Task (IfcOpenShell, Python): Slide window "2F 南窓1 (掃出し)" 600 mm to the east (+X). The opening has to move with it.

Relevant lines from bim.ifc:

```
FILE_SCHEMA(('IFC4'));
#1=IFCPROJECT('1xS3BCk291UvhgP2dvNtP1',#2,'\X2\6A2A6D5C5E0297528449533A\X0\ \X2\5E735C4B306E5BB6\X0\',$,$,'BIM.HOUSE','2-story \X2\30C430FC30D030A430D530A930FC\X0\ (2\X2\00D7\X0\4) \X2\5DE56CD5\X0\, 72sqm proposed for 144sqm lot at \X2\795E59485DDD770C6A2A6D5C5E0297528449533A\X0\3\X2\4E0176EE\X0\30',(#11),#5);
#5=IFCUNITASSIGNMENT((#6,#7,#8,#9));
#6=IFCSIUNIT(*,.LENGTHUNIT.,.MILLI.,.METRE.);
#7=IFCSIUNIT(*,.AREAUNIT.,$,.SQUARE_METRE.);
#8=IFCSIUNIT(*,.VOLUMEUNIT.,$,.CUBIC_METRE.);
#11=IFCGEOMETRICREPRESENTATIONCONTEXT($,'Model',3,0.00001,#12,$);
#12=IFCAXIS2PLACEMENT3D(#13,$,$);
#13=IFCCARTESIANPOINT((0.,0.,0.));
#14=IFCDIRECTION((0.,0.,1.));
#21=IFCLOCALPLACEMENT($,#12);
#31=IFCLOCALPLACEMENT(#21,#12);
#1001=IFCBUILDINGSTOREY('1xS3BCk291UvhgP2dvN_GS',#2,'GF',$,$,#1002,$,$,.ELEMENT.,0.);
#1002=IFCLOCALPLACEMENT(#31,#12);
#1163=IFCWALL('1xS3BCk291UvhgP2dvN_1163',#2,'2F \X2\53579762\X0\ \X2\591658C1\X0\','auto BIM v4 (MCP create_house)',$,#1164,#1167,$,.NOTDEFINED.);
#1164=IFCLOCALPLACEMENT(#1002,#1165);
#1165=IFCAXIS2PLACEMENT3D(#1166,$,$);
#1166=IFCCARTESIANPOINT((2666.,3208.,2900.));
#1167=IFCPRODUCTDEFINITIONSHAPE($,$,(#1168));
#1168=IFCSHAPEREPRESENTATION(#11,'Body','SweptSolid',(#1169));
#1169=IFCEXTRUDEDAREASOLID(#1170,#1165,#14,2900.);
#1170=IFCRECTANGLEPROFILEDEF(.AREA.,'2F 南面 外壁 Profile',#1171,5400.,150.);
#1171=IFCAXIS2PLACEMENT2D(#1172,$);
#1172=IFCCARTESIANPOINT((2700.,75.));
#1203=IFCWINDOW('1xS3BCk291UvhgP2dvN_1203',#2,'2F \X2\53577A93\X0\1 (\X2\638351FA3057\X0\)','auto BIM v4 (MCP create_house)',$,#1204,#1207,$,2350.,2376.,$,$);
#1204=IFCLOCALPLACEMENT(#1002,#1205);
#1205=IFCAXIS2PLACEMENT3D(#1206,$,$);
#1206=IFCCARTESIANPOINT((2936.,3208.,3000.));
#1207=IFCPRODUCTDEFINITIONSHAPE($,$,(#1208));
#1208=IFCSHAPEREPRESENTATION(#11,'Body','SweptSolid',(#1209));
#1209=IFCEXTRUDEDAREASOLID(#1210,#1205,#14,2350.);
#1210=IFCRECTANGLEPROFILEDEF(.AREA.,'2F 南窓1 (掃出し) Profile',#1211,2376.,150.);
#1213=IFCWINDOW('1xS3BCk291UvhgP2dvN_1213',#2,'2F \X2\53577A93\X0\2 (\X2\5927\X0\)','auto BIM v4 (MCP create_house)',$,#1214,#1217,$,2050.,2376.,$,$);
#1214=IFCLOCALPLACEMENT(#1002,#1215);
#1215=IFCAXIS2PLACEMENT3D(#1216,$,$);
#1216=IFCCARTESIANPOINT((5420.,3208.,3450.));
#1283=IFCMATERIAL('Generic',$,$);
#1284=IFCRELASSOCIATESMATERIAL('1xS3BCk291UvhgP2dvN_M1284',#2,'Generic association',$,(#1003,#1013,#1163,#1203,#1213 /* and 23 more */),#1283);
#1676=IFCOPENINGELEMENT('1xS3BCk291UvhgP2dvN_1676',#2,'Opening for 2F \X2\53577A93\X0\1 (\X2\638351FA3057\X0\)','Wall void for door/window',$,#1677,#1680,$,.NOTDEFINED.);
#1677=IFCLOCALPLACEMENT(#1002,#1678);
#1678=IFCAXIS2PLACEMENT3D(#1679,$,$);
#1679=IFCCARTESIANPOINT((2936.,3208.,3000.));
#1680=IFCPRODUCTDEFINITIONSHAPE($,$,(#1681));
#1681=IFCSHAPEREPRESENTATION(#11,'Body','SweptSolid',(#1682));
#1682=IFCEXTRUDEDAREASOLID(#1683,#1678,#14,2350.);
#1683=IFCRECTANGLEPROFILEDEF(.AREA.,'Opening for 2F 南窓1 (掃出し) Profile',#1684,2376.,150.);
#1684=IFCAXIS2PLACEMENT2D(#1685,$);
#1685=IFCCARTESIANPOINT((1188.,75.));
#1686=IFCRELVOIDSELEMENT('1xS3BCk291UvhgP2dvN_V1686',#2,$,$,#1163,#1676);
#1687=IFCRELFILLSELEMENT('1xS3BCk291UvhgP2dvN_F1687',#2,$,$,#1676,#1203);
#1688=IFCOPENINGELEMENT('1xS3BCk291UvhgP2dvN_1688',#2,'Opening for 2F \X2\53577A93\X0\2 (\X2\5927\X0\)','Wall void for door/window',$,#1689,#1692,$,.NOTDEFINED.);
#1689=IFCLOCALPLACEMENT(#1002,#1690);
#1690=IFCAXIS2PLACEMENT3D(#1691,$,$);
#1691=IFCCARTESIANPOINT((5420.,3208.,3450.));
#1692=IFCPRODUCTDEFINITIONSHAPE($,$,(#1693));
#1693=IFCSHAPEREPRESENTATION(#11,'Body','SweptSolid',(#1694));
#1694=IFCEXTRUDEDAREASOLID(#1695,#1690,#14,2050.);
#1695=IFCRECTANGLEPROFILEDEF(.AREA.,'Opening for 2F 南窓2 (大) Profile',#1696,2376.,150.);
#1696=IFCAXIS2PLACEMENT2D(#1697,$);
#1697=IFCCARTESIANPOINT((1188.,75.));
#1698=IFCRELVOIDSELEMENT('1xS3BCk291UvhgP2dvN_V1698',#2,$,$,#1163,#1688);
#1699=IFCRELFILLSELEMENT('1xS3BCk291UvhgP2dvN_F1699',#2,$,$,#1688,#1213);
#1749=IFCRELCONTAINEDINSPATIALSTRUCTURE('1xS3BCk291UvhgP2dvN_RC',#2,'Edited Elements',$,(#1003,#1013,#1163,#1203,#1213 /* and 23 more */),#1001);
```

```python
import ifcopenshell
import ifcopenshell.api.geometry
import ifcopenshell.util.placement

model = ifcopenshell.open("bim.ifc")

window = model.by_guid("1xS3BCk291UvhgP2dvN_1203")
opening = window.FillsVoids[0].RelatingOpeningElement
wall = opening.VoidsElements[0].RelatingBuildingElement

wall_matrix = ifcopenshell.util.placement.get_local_placement(wall.ObjectPlacement)
shift = wall_matrix[:3, 0] * 600.0
before = ifcopenshell.util.placement.get_local_placement(window.ObjectPlacement)[:3, 3].copy()

# The window is not placed relative to its opening, so move both.
for product in (opening, window):
    matrix = ifcopenshell.util.placement.get_local_placement(product.ObjectPlacement)
    matrix[:3, 3] += shift
    ifcopenshell.api.geometry.edit_object_placement(model, product=product, matrix=matrix, is_si=False)

after = ifcopenshell.util.placement.get_local_placement(window.ObjectPlacement)[:3, 3]
print("window moved by", (after - before).round(3) + 0.0)

model.write("bim_rev.ifc")
```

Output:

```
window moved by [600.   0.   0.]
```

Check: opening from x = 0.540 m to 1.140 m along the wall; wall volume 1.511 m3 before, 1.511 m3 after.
